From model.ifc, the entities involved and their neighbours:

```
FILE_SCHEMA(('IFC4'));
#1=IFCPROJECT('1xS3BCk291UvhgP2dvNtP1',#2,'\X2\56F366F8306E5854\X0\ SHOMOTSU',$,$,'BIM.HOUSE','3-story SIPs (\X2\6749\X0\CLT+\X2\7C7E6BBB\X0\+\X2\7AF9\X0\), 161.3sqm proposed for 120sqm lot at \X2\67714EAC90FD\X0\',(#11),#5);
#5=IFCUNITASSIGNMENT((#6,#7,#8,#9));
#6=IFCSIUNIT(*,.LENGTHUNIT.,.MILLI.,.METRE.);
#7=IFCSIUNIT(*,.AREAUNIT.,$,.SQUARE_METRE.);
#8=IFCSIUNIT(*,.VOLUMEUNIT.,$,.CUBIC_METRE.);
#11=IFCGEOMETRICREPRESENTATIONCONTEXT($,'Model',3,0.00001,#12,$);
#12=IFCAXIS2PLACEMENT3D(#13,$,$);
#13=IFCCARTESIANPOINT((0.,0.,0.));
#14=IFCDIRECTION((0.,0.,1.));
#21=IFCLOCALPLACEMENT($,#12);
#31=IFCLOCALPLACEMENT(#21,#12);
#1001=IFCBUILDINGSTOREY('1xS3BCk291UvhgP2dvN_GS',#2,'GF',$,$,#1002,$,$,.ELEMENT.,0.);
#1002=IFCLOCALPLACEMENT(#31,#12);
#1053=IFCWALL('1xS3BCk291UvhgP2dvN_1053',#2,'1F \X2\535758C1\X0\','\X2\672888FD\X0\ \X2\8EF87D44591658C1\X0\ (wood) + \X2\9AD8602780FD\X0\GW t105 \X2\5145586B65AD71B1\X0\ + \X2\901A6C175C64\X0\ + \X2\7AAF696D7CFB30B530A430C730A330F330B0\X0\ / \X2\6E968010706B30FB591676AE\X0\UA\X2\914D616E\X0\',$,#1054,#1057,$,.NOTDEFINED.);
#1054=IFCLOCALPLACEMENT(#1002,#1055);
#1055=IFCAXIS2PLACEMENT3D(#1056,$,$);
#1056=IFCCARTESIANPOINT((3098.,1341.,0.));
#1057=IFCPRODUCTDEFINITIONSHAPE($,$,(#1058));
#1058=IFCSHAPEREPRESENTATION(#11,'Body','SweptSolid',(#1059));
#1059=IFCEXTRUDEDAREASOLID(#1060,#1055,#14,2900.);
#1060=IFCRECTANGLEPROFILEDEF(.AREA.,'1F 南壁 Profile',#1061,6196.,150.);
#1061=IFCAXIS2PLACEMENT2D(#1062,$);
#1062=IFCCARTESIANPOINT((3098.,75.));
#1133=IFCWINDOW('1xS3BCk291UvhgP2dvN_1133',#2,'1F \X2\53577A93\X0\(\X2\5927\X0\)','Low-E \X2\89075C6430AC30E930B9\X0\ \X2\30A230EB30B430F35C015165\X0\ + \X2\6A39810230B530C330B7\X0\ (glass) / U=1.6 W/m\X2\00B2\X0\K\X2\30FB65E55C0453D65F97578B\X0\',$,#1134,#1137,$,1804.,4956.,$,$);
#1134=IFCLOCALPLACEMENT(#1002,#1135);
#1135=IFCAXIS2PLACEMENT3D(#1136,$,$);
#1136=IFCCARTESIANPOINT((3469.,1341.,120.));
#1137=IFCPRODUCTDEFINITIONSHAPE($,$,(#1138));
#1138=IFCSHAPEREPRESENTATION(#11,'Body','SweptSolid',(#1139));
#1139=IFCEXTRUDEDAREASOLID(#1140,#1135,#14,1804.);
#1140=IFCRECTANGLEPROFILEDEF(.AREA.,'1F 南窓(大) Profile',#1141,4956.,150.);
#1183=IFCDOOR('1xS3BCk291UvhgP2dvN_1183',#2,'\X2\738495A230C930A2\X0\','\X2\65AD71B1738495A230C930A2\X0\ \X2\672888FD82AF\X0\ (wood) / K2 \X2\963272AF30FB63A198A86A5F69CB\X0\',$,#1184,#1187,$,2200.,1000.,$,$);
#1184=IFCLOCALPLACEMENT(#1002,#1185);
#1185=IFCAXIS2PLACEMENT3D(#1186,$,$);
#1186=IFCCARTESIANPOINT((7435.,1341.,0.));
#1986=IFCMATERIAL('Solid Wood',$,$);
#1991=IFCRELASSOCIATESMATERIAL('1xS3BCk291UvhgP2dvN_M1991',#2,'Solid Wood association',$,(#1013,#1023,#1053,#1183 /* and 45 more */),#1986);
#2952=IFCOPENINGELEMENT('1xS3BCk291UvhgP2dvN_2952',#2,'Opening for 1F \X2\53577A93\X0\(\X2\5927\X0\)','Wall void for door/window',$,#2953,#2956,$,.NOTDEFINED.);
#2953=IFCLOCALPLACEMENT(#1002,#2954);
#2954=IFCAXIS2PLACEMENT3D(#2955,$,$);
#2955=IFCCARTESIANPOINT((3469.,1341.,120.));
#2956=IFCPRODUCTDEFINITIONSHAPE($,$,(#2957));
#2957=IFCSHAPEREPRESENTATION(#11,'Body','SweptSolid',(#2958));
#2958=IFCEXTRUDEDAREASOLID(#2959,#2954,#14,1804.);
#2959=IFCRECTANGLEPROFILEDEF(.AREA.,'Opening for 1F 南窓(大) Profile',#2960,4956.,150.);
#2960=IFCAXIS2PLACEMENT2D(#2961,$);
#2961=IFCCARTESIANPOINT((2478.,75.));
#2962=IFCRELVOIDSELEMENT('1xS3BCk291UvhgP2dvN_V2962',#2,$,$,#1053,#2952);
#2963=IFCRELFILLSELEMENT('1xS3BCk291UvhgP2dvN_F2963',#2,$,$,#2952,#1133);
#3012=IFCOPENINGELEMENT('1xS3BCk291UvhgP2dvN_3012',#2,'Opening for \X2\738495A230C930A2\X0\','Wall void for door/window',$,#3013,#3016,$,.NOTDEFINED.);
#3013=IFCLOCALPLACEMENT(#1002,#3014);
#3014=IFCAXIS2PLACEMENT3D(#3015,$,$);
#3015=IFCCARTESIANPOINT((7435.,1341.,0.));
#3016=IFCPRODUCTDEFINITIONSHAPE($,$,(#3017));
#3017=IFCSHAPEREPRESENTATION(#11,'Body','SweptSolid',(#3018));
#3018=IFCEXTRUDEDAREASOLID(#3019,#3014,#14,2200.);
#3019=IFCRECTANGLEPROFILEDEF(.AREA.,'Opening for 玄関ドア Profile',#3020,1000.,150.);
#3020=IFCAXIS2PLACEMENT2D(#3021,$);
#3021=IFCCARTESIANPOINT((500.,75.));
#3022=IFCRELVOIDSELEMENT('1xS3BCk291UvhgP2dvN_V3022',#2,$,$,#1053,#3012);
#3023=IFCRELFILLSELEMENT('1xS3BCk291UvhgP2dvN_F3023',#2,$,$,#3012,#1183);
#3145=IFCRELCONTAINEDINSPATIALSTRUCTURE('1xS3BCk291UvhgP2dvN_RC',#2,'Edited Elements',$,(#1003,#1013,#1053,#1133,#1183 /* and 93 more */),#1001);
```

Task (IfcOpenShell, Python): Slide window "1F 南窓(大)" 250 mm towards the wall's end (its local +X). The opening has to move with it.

```python
import ifcopenshell
import ifcopenshell.api.geometry
import ifcopenshell.util.placement
import ifcopenshell.util.unit

model = ifcopenshell.open("model.ifc")
unit_scale = ifcopenshell.util.unit.calculate_unit_scale(model)

window = model.by_guid("1xS3BCk291UvhgP2dvN_1133")
opening = window.FillsVoids[0].RelatingOpeningElement
wall = opening.VoidsElements[0].RelatingBuildingElement

wall_matrix = ifcopenshell.util.placement.get_local_placement(wall.ObjectPlacement)
shift = wall_matrix[:3, 0] * 0.25 / unit_scale
before = ifcopenshell.util.placement.get_local_placement(window.ObjectPlacement)[:3, 3].copy()

# The window is not placed relative to its opening, so move both.
for product in (opening, window):
    matrix = ifcopenshell.util.placement.get_local_placement(product.ObjectPlacement)
    matrix[:3, 3] += shift
    ifcopenshell.api.geometry.edit_object_placement(model, product=product, matrix=matrix, is_si=False)

after = ifcopenshell.util.placement.get_local_placement(window.ObjectPlacement)[:3, 3]
print("window moved by", (after - before).round(3) + 0.0)

model.write("model_rev.ifc")
```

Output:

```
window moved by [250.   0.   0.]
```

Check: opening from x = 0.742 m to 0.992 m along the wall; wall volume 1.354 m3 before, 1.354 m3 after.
